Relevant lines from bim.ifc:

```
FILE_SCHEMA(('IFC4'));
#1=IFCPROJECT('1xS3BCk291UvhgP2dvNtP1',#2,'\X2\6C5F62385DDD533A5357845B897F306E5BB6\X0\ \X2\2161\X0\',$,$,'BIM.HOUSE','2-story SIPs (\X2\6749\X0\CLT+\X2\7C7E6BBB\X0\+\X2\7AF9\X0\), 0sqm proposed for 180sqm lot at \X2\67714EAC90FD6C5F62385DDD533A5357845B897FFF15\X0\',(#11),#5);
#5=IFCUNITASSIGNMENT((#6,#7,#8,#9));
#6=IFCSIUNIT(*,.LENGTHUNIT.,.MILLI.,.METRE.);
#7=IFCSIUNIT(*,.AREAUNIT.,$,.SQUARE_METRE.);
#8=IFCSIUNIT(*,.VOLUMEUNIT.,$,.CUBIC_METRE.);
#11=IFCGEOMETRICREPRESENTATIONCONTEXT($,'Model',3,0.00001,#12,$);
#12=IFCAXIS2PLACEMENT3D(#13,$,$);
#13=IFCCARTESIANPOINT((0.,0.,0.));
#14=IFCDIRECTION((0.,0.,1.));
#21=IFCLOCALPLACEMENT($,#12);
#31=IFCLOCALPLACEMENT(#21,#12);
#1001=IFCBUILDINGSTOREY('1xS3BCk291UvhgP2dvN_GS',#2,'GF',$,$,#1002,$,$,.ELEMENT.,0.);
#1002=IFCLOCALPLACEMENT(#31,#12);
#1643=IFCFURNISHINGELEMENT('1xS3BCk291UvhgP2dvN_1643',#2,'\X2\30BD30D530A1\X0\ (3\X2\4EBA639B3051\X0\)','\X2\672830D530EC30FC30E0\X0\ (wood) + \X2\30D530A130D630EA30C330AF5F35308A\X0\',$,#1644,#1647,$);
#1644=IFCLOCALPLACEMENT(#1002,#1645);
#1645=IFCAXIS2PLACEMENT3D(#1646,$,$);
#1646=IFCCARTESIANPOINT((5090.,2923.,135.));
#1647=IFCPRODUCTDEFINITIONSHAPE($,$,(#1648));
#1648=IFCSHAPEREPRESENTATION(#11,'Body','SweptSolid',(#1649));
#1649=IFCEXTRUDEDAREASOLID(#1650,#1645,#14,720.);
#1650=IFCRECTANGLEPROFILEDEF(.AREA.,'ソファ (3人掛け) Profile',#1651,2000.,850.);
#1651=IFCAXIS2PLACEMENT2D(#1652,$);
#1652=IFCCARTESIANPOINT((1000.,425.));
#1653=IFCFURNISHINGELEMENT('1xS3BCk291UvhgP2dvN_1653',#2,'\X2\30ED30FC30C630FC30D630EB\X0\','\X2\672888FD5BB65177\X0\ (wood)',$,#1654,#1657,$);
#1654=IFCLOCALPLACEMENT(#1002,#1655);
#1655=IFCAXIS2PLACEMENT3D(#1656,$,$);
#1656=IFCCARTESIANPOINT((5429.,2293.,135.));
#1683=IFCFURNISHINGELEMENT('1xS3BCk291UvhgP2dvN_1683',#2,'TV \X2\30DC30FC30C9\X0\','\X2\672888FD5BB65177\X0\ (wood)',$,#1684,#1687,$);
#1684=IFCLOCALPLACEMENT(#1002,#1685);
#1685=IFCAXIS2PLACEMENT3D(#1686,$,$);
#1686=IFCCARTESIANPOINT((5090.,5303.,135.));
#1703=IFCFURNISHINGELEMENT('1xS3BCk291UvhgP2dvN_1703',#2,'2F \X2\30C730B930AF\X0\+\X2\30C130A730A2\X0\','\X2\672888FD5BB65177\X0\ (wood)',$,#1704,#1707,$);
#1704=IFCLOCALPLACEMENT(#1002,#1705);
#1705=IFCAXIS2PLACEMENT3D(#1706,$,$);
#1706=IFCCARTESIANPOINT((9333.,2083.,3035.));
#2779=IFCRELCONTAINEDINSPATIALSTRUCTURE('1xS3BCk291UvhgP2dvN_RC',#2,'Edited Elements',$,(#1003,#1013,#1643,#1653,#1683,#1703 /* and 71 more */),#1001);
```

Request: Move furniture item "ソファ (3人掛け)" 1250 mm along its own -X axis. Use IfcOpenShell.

```python
import ifcopenshell
import ifcopenshell.api.geometry
import ifcopenshell.util.placement
import ifcopenshell.util.unit

model = ifcopenshell.open("bim.ifc")
unit_scale = ifcopenshell.util.unit.calculate_unit_scale(model)

item = model.by_guid("1xS3BCk291UvhgP2dvN_1643")
matrix = ifcopenshell.util.placement.get_local_placement(item.ObjectPlacement)
matrix[:3, 3] -= matrix[:3, 0] * 1.25 / unit_scale
ifcopenshell.api.geometry.edit_object_placement(model, product=item, matrix=matrix, is_si=False)

print(ifcopenshell.util.placement.get_local_placement(item.ObjectPlacement).round(3) + 0.0)

model.write("bim_updated.ifc")
```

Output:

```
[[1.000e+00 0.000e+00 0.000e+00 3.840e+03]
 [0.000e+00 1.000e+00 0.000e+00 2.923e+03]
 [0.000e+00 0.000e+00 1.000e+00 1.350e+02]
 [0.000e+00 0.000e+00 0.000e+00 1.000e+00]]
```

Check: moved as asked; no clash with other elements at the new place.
